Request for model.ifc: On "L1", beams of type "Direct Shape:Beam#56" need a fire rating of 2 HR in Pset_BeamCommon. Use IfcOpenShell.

First a look at what the model holds.

```python
import ifcopenshell
import ifcopenshell.util.element

model = ifcopenshell.open("model.ifc")
print(model.schema)
storey = next(s for s in model.by_type("IfcBuildingStorey") if s.Name == "L1")
beams = [e for e in ifcopenshell.util.element.get_decomposition(storey) if e.is_a("IfcBeam")]
seen = {}
for e in beams:
    element_type = ifcopenshell.util.element.get_type(e)
    key = (element_type.Name if element_type != e and element_type else None, ifcopenshell.util.element.get_pset(e, "Pset_BeamCommon", "FireRating"))
    seen[key] = seen.get(key, 0) + 1
for (name, value), count in sorted(seen.items(), key=str):
    print(count, "x", name, "|", value)
```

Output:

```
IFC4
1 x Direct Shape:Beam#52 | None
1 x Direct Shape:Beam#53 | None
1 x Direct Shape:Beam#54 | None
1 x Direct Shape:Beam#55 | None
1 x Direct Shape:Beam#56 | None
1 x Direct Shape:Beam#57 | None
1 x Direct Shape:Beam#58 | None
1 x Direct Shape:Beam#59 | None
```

```python
import ifcopenshell
import ifcopenshell.api.pset
import ifcopenshell.util.element

model = ifcopenshell.open("model.ifc")

storey = next(s for s in model.by_type("IfcBuildingStorey") if s.Name == "L1")
beams = [e for e in ifcopenshell.util.element.get_decomposition(storey) if e.is_a("IfcBeam")]

count = 0
for e in beams:
    element_type = ifcopenshell.util.element.get_type(e)
    if element_type in (None, e) or element_type.Name != "Direct Shape:Beam#56":
        continue
    # add_pset returns the element's existing set when there is one.
    pset = ifcopenshell.api.pset.add_pset(model, product=e, name="Pset_BeamCommon")
    ifcopenshell.api.pset.edit_pset(model, pset=pset, properties={"FireRating": "2 HR"})
    count += 1

print(count, "beams updated")

model.write("model_edited.ifc")
```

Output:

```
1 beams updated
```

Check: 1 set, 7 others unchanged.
